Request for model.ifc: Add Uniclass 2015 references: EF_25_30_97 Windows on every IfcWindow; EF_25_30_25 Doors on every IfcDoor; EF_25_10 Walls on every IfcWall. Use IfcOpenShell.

First a look at what the model holds.

```python
import ifcopenshell

model = ifcopenshell.open("model.ifc")
print(model.schema)
print("classifications:", [c.Name for c in model.by_type("IfcClassification")])
for ifc_class in ("IfcDoor", "IfcRoof", "IfcStair", "IfcWall", "IfcWindow"):
    print(ifc_class, len(model.by_type(ifc_class)))
```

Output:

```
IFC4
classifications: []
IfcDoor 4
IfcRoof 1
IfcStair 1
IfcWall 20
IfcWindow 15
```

```python
import ifcopenshell
import ifcopenshell.api.classification

model = ifcopenshell.open("model.ifc")

system = ifcopenshell.api.classification.add_classification(model, classification="Uniclass 2015")

codes = {
    "IfcWindow": ("EF_25_30_97", "Windows"),
    "IfcDoor": ("EF_25_30_25", "Doors"),
    "IfcWall": ("EF_25_10", "Walls"),
}
for ifc_class, (code, name) in codes.items():
    products = model.by_type(ifc_class)
    ifcopenshell.api.classification.add_reference(
        model, products=products, classification=system, identification=code, name=name
    )
    print(code, len(products))

model.write("model_rev.ifc")
```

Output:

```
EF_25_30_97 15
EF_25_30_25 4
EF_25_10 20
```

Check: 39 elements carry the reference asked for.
